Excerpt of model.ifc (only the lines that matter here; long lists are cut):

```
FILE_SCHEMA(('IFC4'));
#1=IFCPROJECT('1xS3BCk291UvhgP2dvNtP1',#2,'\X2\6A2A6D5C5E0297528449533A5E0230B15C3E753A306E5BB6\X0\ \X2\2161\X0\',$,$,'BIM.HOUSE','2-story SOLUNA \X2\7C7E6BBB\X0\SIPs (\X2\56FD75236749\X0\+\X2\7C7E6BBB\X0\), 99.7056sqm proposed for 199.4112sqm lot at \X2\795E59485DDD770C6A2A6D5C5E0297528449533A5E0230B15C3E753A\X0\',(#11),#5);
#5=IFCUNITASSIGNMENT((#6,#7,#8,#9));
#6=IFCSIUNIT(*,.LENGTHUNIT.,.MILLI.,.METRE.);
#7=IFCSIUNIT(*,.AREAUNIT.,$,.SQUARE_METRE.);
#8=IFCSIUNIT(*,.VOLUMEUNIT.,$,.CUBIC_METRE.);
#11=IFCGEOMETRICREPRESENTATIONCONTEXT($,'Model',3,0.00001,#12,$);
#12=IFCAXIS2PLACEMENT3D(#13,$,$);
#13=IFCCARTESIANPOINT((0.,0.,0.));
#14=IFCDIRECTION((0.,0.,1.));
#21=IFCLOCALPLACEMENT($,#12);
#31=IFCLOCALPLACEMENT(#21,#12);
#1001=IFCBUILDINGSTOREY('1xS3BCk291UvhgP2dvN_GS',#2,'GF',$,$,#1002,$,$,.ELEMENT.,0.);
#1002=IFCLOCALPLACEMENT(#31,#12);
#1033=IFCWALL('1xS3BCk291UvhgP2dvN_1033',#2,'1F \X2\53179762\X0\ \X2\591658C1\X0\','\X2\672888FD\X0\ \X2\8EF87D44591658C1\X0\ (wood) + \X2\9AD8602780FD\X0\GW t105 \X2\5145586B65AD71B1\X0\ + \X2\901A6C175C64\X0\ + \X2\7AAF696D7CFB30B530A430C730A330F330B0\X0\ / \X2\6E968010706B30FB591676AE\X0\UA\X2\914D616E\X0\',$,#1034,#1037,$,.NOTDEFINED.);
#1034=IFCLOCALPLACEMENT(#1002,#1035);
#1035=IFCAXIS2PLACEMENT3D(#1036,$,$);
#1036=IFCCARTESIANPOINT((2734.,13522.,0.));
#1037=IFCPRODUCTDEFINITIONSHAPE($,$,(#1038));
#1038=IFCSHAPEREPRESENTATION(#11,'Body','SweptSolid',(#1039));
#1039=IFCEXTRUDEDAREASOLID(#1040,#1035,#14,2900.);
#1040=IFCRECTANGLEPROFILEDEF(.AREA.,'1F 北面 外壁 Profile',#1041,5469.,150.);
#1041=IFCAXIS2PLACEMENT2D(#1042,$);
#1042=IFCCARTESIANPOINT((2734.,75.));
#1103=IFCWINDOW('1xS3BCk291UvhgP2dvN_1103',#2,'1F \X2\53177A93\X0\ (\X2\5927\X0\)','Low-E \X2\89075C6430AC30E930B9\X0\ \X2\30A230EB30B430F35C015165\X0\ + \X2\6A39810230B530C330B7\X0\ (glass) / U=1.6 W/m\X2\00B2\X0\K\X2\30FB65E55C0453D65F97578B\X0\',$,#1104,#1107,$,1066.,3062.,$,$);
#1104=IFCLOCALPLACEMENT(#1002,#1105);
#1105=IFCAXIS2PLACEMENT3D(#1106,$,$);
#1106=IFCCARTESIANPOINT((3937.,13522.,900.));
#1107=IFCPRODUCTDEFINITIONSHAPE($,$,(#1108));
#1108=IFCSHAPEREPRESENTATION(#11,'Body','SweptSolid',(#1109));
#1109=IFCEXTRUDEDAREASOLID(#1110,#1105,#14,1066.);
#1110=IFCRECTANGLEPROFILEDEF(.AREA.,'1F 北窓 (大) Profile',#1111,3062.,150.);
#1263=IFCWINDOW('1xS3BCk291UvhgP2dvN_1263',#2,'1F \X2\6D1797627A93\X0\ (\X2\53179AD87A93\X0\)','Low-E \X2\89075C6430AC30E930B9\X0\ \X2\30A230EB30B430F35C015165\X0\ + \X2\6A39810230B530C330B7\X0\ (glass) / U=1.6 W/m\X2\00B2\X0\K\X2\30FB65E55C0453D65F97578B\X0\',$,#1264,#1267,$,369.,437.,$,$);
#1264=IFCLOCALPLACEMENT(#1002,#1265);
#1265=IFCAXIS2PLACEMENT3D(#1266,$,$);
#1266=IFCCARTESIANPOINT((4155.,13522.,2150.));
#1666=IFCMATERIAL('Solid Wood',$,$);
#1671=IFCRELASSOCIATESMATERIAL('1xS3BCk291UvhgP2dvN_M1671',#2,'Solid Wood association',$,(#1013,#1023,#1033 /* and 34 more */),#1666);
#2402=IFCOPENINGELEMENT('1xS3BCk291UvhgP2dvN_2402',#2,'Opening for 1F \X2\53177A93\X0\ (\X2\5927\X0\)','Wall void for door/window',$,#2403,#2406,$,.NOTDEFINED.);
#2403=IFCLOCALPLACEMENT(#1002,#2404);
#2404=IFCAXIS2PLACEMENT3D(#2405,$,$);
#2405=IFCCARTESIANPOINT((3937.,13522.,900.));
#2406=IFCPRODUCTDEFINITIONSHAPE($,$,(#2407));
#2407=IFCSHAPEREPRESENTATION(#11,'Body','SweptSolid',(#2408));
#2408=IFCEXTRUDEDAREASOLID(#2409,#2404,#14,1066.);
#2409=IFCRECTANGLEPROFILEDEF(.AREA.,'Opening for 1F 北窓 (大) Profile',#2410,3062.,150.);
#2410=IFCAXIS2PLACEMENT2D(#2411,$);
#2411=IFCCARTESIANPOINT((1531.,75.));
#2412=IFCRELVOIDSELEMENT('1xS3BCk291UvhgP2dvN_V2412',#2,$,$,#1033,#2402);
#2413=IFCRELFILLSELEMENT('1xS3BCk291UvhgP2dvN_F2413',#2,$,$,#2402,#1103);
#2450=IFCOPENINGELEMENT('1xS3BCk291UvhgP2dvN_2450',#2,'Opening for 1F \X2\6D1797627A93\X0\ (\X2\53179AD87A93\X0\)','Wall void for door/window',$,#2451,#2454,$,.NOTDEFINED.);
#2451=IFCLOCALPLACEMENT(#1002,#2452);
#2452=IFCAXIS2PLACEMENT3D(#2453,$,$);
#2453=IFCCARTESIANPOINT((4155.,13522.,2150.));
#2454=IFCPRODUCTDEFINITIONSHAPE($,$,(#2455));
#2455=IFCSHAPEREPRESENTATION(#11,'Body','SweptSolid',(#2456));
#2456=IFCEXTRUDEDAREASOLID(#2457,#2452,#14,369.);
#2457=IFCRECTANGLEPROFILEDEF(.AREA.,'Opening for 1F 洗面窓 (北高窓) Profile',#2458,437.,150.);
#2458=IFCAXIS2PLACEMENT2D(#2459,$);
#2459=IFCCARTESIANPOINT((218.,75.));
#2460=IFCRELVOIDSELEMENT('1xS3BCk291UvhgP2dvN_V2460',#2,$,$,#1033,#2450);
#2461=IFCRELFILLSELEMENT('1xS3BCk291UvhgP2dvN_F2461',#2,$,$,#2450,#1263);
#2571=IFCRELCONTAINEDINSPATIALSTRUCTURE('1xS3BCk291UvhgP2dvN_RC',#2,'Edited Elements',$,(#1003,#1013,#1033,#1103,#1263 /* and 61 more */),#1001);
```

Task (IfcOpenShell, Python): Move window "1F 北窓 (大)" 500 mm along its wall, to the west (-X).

```python
import ifcopenshell
import ifcopenshell.api.geometry
import ifcopenshell.util.placement
import ifcopenshell.util.unit

model = ifcopenshell.open("model.ifc")
unit_scale = ifcopenshell.util.unit.calculate_unit_scale(model)

window = model.by_guid("1xS3BCk291UvhgP2dvN_1103")
opening = window.FillsVoids[0].RelatingOpeningElement
wall = opening.VoidsElements[0].RelatingBuildingElement

wall_matrix = ifcopenshell.util.placement.get_local_placement(wall.ObjectPlacement)
shift = wall_matrix[:3, 0] * -0.5 / unit_scale
before = ifcopenshell.util.placement.get_local_placement(window.ObjectPlacement)[:3, 3].copy()

# The window is not placed relative to its opening, so move both.
for product in (opening, window):
    matrix = ifcopenshell.util.placement.get_local_placement(product.ObjectPlacement)
    matrix[:3, 3] += shift
    ifcopenshell.api.geometry.edit_object_placement(model, product=product, matrix=matrix, is_si=False)

after = ifcopenshell.util.placement.get_local_placement(window.ObjectPlacement)[:3, 3]
print("window moved by", (after - before).round(3) + 0.0)

model.write("model-out.ifc")
```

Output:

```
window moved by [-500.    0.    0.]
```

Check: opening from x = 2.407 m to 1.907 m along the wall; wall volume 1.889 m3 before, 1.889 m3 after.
